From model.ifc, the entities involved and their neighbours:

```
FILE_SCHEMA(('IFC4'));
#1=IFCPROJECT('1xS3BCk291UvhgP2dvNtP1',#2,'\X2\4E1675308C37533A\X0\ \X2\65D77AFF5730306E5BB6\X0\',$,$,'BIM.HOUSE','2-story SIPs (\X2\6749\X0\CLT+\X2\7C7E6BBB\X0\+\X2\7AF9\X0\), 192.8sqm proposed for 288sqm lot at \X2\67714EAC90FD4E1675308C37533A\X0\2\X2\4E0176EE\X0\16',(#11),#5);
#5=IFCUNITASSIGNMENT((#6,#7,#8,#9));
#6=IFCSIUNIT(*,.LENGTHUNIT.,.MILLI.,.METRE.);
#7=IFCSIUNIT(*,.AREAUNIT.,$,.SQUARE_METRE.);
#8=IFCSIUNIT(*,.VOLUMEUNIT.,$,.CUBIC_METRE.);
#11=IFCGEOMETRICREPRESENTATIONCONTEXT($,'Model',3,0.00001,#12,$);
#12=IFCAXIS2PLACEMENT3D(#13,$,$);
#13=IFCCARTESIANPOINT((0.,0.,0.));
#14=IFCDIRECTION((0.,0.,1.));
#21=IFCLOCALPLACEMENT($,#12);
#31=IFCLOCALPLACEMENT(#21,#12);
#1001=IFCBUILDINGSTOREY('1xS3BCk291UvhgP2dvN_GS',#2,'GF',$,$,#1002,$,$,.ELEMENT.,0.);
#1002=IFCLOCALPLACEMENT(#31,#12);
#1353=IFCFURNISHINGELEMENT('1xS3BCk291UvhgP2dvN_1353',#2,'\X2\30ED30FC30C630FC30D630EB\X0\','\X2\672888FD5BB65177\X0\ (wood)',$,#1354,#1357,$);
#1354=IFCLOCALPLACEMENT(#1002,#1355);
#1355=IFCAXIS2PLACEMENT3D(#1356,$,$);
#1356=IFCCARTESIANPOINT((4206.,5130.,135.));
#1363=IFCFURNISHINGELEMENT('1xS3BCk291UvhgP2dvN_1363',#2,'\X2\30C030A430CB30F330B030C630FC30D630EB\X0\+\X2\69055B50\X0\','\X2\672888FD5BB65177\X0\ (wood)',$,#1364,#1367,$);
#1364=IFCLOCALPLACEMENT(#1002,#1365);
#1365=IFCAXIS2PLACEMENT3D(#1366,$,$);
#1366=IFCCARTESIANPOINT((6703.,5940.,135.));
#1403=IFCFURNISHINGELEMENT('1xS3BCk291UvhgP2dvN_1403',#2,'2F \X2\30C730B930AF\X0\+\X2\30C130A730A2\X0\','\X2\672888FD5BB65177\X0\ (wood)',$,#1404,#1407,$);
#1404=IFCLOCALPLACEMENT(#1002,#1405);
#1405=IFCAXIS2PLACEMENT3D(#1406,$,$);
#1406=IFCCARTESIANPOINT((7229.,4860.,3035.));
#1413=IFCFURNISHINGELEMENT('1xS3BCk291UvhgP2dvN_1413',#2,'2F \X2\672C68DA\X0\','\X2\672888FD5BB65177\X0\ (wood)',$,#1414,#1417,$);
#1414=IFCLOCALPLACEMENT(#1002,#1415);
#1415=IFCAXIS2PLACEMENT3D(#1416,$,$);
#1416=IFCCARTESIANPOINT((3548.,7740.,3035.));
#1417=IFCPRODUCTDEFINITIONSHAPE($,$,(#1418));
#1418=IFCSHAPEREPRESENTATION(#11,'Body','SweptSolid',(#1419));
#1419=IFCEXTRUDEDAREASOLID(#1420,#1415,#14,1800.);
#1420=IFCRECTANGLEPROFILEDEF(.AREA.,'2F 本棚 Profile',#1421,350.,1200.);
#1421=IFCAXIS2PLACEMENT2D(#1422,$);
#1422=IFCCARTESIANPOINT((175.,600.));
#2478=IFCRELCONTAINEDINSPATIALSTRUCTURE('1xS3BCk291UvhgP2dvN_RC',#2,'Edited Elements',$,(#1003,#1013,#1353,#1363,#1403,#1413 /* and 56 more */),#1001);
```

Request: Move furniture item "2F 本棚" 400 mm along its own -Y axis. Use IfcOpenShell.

```python
import ifcopenshell
import ifcopenshell.api.geometry
import ifcopenshell.util.placement
import ifcopenshell.util.unit

model = ifcopenshell.open("model.ifc")
unit_scale = ifcopenshell.util.unit.calculate_unit_scale(model)

item = model.by_id(1413)
matrix = ifcopenshell.util.placement.get_local_placement(item.ObjectPlacement)
matrix[:3, 3] -= matrix[:3, 1] * 0.4 / unit_scale
ifcopenshell.api.geometry.edit_object_placement(model, product=item, matrix=matrix, is_si=False)

print(ifcopenshell.util.placement.get_local_placement(item.ObjectPlacement).round(3) + 0.0)

model.write("model_updated.ifc")
```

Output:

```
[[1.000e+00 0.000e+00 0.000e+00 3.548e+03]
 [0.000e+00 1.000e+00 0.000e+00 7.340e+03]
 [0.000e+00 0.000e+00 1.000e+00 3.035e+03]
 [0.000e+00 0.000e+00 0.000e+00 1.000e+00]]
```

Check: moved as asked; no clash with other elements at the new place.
